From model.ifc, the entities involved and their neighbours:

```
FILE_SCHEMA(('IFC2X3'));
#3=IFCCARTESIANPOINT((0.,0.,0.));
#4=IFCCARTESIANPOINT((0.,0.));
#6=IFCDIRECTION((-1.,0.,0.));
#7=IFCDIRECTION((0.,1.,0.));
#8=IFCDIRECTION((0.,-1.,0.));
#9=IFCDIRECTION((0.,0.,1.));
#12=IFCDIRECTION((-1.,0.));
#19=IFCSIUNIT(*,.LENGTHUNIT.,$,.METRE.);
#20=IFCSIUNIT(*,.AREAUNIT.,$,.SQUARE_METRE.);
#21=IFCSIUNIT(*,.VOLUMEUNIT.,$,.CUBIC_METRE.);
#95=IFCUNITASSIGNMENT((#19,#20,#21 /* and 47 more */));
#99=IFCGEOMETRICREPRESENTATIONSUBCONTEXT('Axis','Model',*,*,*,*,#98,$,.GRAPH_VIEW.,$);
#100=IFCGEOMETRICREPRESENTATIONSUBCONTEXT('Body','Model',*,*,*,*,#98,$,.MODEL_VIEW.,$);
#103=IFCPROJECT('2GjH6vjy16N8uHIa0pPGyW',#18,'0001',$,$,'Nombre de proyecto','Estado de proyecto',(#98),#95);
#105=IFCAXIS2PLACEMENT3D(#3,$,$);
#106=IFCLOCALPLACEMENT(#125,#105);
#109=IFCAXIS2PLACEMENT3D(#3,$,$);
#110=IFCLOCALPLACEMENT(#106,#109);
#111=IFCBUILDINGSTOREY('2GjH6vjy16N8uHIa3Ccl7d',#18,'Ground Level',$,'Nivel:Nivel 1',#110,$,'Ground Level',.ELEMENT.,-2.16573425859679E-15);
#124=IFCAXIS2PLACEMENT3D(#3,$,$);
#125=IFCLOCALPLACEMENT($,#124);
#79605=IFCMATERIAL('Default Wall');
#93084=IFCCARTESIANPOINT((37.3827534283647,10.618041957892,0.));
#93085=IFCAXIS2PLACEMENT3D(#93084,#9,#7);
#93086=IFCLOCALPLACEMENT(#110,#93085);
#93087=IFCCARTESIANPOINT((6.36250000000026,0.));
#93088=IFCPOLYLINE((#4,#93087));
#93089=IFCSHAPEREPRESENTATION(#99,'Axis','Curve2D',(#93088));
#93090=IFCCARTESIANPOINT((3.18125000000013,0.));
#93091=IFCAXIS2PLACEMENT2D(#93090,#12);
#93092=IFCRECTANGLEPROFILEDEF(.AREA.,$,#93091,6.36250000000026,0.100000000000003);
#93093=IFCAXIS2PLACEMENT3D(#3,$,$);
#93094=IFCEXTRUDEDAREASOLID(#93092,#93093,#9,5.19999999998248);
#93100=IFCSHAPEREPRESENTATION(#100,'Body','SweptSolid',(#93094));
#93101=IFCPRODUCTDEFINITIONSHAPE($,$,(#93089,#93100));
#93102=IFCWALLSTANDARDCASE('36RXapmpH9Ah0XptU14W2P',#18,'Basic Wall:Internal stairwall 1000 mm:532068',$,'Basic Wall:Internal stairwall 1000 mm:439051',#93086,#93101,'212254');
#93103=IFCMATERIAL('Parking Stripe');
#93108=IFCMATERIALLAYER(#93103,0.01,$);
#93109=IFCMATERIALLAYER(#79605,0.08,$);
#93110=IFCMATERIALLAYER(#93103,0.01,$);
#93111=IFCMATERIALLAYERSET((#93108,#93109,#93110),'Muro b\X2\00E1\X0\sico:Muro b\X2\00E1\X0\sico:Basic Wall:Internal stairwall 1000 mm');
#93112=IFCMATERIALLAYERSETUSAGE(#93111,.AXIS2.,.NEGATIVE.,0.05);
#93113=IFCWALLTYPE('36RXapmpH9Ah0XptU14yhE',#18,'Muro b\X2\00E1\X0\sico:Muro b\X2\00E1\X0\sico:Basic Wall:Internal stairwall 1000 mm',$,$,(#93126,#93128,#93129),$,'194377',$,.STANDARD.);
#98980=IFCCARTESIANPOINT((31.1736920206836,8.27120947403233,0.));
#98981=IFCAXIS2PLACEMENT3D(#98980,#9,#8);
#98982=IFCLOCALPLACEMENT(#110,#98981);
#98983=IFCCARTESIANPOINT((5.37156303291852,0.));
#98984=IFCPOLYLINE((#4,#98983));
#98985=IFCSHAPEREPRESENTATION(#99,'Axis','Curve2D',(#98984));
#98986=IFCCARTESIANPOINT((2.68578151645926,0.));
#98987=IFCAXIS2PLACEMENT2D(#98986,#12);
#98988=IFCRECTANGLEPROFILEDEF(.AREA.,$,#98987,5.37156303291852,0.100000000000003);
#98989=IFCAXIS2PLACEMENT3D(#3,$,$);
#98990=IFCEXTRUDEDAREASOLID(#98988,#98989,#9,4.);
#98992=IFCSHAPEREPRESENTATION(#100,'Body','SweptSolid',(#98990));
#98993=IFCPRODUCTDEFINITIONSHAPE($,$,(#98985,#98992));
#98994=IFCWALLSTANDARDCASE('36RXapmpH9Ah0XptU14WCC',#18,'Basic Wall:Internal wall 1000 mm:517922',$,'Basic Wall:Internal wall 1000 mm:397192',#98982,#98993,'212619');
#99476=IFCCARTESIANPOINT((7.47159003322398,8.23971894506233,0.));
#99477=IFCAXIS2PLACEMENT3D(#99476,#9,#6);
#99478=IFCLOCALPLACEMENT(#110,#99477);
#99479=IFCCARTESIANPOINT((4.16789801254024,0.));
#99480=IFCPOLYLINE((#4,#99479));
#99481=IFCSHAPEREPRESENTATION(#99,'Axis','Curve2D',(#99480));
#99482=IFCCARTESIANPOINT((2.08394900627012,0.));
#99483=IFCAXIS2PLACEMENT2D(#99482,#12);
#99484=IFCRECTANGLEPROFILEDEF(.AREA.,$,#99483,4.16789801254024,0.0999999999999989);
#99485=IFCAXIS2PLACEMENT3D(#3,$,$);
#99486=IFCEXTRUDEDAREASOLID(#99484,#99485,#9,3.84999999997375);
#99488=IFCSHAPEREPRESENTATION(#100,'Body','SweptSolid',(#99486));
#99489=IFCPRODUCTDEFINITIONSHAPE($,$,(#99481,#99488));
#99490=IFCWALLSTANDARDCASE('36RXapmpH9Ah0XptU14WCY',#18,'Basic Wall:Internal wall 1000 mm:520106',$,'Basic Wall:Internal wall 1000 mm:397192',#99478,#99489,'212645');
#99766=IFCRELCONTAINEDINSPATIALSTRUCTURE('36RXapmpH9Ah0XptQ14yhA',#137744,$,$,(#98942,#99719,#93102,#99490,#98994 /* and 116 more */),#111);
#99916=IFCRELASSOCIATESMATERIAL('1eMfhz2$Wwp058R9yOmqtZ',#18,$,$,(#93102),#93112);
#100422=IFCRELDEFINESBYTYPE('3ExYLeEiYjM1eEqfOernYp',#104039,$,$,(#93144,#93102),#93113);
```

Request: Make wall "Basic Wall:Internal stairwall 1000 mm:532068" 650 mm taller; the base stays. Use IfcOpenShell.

```python
import ifcopenshell
import ifcopenshell.geom
import ifcopenshell.util.representation
import ifcopenshell.util.shape

model = ifcopenshell.open("model.ifc")
settings = ifcopenshell.geom.settings()


def volume(element):
    """Net volume in cubic metres, openings subtracted."""
    shape = ifcopenshell.geom.create_shape(settings, element)
    return ifcopenshell.util.shape.get_volume(shape.geometry)


wall = model.by_guid("36RXapmpH9Ah0XptU14W2P")
before = volume(wall)

body = ifcopenshell.util.representation.get_representation(wall, "Model", "Body")
solid = body.Items[0]
old_height = solid.Depth
solid.Depth += 0.65
after = volume(wall)

print(f"height {old_height:g} -> {solid.Depth:g}, volume {before:.3f} -> {after:.3f} m3")

model.write("model_rev.ifc")
```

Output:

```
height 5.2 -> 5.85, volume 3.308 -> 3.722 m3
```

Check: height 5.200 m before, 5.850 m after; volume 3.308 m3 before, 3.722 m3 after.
